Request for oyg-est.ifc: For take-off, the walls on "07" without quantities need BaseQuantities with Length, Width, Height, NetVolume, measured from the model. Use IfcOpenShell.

First a look at what the model holds.

```python
import ifcopenshell
import ifcopenshell.util.element
import ifcopenshell.util.unit

model = ifcopenshell.open("oyg-est.ifc")
print(model.schema)
for unit_type in ("LENGTHUNIT", "AREAUNIT", "VOLUMEUNIT"):
    print(unit_type, ifcopenshell.util.unit.calculate_unit_scale(model, unit_type))
storey = next(s for s in model.by_type("IfcBuildingStorey") if s.Name == "07")
walls = [e for e in ifcopenshell.util.element.get_decomposition(storey) if e.is_a("IfcWall")]
for e in sorted(walls, key=lambda e: e.id()):
    print(e.id(), e.is_a(), e.Name, list(ifcopenshell.util.element.get_psets(e, qtos_only=True)), sep=" | ")
```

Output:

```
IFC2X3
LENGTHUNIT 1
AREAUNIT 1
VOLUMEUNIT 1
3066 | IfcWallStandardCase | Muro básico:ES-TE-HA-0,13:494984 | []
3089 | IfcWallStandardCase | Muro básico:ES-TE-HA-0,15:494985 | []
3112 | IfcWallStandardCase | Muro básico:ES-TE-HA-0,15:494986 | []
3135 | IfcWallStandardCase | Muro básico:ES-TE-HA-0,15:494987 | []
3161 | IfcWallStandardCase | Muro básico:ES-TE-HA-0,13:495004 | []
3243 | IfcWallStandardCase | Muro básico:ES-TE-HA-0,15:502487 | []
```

```python
import ifcopenshell
import ifcopenshell.api.pset
import ifcopenshell.geom
import ifcopenshell.util.element
import ifcopenshell.util.shape
import ifcopenshell.util.unit

model = ifcopenshell.open("oyg-est.ifc")
unit_scale = ifcopenshell.util.unit.calculate_unit_scale(model)
volume_scale = ifcopenshell.util.unit.calculate_unit_scale(model, "VOLUMEUNIT")
settings = ifcopenshell.geom.settings()

storey = next(s for s in model.by_type("IfcBuildingStorey") if s.Name == "07")
walls = [e for e in ifcopenshell.util.element.get_decomposition(storey) if e.is_a("IfcWall")]

for e in sorted(walls, key=lambda e: e.id()):
    if ifcopenshell.util.element.get_psets(e, qtos_only=True, should_inherit=False):
        continue
    # Geometry comes back in metres, in the element's own axes.
    shape = ifcopenshell.geom.create_shape(settings, e)
    values = {
        "Length": ifcopenshell.util.shape.get_x(shape.geometry) / unit_scale,
        "Width": ifcopenshell.util.shape.get_y(shape.geometry) / unit_scale,
        "Height": ifcopenshell.util.shape.get_z(shape.geometry) / unit_scale,
        "NetVolume": ifcopenshell.util.shape.get_volume(shape.geometry) / volume_scale,
    }
    qto = ifcopenshell.api.pset.add_qto(model, product=e, name="BaseQuantities")
    ifcopenshell.api.pset.edit_qto(model, qto=qto, properties=values)
    print(e.id(), {k: round(v, 3) for k, v in values.items()})

model.write("oyg-est_rev.ifc")
```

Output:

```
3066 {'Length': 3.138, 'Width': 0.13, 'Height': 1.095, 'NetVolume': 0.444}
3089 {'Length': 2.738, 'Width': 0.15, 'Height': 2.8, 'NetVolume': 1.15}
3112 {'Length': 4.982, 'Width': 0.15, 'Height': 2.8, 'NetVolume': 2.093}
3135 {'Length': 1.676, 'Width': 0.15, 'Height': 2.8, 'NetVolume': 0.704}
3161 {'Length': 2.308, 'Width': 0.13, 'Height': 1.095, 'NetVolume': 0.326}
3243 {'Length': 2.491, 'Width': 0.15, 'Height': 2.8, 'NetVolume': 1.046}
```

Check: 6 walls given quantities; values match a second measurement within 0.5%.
